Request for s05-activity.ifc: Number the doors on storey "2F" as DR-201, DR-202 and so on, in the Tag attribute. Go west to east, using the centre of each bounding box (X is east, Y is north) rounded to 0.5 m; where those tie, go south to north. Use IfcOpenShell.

First a look at what the model holds.

```python
import ifcopenshell
import ifcopenshell.util.element
import ifcopenshell.util.placement

model = ifcopenshell.open("s05-activity.ifc")
print(model.schema)
storey = next(s for s in model.by_type("IfcBuildingStorey") if s.Name == "2F")
doors = [e for e in ifcopenshell.util.element.get_decomposition(storey) if e.is_a("IfcDoor")]
for e in sorted(doors, key=lambda e: e.id()):
    origin = ifcopenshell.util.placement.get_local_placement(e.ObjectPlacement)[:3, 3]
    print(e.id(), e.Tag, e.Name, origin.round(2) + 0.0, sep=" | ")
```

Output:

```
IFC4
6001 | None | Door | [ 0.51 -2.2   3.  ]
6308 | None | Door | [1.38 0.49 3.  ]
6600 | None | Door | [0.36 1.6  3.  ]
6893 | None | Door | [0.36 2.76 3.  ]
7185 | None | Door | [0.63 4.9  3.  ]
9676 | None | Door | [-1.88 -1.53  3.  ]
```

```python
import ifcopenshell
import ifcopenshell.geom
import ifcopenshell.util.element
import ifcopenshell.util.shape

model = ifcopenshell.open("s05-activity.ifc")
settings = ifcopenshell.geom.settings()
settings.set("use-world-coords", True)


def centre(element):
    shape = ifcopenshell.geom.create_shape(settings, element)
    return ifcopenshell.util.shape.get_bbox_centroid(shape.geometry)


storey = next(s for s in model.by_type("IfcBuildingStorey") if s.Name == "2F")
doors = [e for e in ifcopenshell.util.element.get_decomposition(storey) if e.is_a("IfcDoor")]

# Insertion points can sit at a corner or the storey origin, so sort by the geometry (in metres).
centres = {e: centre(e) for e in doors}
doors.sort(key=lambda e: (round(centres[e][0] / 0.5), centres[e][1]))

for i, e in enumerate(doors, start=1):
    number = f"DR-2{i:02d}"
    e.Tag = number
    print(e.id(), number)

model.write("s05-activity_v2.ifc")
```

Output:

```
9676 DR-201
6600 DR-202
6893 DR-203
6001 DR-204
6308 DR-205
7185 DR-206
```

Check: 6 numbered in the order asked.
